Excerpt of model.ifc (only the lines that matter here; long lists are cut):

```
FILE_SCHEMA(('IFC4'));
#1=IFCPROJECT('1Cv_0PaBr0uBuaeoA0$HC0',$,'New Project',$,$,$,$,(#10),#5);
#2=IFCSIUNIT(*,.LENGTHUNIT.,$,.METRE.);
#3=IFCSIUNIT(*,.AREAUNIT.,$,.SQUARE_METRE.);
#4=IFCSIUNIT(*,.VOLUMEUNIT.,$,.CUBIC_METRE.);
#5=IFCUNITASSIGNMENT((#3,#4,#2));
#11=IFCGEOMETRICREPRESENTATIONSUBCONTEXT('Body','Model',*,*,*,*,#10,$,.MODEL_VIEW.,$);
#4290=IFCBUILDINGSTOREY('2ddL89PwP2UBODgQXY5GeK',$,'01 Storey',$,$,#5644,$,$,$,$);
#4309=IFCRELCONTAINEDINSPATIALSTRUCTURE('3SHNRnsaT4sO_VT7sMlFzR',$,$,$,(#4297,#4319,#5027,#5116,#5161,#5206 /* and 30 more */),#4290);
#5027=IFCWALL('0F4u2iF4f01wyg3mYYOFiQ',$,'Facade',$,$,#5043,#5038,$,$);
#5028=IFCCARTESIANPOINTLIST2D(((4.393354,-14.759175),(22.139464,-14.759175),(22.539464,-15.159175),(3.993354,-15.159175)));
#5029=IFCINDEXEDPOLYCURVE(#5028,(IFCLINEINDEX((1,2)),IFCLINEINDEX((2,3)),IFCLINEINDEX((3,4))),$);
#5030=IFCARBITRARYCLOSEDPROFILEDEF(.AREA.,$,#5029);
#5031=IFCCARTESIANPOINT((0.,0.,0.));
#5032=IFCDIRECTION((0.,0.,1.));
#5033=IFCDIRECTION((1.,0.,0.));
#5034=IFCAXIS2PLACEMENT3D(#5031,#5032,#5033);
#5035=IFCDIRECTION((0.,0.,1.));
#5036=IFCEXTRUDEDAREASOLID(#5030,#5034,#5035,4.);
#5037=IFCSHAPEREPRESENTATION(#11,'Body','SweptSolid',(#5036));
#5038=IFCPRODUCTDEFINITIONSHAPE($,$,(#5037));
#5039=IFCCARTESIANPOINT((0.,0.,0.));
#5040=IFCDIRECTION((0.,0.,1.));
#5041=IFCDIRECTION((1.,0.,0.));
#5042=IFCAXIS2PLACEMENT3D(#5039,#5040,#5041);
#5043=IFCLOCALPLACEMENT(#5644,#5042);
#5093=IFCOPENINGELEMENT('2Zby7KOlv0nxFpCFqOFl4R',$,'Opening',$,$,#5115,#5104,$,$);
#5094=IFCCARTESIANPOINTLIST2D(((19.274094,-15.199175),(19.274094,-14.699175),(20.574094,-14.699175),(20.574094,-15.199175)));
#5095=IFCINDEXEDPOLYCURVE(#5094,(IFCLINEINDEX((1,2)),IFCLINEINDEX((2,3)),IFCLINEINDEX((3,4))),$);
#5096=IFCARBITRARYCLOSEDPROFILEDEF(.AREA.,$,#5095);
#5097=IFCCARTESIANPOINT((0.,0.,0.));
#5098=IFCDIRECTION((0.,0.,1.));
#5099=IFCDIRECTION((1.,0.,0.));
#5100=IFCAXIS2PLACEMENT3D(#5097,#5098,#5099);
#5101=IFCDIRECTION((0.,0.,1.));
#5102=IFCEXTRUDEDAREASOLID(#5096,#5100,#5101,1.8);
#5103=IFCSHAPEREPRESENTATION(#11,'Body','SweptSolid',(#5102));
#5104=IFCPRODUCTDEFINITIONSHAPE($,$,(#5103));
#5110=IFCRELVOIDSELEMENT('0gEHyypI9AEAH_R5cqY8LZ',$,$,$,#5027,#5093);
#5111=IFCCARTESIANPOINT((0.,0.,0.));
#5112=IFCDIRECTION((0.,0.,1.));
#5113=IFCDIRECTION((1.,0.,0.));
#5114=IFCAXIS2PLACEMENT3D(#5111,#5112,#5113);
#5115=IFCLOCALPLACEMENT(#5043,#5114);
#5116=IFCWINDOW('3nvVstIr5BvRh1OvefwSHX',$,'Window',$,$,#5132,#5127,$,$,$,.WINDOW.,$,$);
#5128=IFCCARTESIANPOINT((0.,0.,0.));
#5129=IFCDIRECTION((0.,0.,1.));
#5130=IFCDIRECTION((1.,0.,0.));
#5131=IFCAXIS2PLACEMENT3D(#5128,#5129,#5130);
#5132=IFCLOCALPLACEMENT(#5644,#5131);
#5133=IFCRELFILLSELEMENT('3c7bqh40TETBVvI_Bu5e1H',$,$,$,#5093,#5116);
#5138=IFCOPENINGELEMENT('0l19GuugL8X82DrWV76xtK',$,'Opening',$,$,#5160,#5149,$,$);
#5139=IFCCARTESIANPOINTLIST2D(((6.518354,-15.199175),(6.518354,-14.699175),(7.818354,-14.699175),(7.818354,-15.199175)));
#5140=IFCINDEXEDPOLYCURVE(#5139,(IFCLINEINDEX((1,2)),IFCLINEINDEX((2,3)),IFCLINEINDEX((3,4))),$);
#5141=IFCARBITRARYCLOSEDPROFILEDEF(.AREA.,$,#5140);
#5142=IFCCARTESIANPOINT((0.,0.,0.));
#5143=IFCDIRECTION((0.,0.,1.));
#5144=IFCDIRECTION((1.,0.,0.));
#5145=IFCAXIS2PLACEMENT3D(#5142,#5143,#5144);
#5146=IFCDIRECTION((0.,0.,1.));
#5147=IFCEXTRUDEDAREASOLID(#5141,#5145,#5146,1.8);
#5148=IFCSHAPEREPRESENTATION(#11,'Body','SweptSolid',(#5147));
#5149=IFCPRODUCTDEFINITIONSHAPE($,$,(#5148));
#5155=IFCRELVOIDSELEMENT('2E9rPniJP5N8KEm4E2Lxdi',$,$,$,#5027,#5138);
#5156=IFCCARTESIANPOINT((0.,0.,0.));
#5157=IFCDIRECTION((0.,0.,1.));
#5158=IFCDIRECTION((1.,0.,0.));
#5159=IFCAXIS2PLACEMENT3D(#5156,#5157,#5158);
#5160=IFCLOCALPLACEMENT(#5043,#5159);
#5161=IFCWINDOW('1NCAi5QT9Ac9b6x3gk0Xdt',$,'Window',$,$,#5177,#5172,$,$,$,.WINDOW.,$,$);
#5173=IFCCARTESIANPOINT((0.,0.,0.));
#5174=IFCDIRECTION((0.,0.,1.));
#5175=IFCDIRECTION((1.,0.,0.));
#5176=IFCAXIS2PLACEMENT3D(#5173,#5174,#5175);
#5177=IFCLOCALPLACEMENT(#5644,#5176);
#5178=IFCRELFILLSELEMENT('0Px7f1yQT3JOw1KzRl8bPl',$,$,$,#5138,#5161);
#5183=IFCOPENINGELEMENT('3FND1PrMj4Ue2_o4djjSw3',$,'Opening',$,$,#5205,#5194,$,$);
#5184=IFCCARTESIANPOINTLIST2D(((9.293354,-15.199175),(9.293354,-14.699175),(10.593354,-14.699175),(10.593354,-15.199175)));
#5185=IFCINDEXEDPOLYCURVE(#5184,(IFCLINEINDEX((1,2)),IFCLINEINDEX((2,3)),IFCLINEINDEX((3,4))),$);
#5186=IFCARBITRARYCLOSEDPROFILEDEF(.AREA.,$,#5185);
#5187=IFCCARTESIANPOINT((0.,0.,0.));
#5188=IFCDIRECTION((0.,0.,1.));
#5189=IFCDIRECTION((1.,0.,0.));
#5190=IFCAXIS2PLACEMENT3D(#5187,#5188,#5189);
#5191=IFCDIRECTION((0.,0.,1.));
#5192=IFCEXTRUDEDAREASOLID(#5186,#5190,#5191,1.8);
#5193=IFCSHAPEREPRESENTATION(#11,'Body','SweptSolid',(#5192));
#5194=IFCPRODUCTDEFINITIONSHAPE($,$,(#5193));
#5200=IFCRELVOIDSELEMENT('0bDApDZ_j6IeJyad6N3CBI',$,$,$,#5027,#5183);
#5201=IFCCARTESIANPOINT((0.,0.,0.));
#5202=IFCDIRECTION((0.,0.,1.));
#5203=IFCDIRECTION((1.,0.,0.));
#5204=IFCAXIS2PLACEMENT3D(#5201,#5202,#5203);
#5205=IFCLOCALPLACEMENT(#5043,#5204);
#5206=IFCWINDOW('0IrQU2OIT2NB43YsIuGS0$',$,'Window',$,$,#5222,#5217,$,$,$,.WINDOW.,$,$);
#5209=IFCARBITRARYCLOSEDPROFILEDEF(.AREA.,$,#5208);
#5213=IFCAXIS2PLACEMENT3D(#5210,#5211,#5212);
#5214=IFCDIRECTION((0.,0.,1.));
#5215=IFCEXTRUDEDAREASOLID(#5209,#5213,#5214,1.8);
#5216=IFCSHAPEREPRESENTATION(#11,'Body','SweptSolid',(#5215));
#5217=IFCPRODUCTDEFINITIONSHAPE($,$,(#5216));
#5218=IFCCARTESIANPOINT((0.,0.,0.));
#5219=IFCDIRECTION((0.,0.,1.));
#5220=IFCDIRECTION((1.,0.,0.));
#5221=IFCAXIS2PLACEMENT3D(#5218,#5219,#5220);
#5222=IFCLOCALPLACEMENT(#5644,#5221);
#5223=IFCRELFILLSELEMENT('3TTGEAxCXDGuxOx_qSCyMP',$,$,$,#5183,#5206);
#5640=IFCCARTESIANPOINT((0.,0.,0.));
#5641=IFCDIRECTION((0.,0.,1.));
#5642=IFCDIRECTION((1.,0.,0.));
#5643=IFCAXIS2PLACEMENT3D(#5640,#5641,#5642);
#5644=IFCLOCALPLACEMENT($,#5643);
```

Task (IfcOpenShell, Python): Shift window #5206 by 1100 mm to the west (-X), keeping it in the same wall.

```python
import ifcopenshell
import ifcopenshell.api.geometry
import ifcopenshell.util.placement

model = ifcopenshell.open("model.ifc")

window = model.by_guid("0IrQU2OIT2NB43YsIuGS0$")
opening = window.FillsVoids[0].RelatingOpeningElement
wall = opening.VoidsElements[0].RelatingBuildingElement

wall_matrix = ifcopenshell.util.placement.get_local_placement(wall.ObjectPlacement)
shift = wall_matrix[:3, 0] * -1.1
before = ifcopenshell.util.placement.get_local_placement(window.ObjectPlacement)[:3, 3].copy()

# The window is not placed relative to its opening, so move both.
for product in (opening, window):
    matrix = ifcopenshell.util.placement.get_local_placement(product.ObjectPlacement)
    matrix[:3, 3] += shift
    ifcopenshell.api.geometry.edit_object_placement(model, product=product, matrix=matrix, is_si=False)

after = ifcopenshell.util.placement.get_local_placement(window.ObjectPlacement)[:3, 3]
print("window moved by", (after - before).round(3) + 0.0)

model.write("model_v2.ifc")
```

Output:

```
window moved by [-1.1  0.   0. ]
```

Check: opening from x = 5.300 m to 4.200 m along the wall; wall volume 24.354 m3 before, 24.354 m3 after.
